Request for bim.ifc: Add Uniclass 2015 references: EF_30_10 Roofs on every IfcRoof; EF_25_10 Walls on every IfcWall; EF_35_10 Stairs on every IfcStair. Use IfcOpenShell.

First a look at what the model holds.

```python
import ifcopenshell

model = ifcopenshell.open("bim.ifc")
print(model.schema)
print("classifications:", [c.Name for c in model.by_type("IfcClassification")])
for ifc_class in ("IfcDoor", "IfcRoof", "IfcStair", "IfcWall", "IfcWindow"):
    print(ifc_class, len(model.by_type(ifc_class)))
```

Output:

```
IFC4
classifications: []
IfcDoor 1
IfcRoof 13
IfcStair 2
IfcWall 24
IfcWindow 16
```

```python
import ifcopenshell
import ifcopenshell.api.classification

model = ifcopenshell.open("bim.ifc")

system = ifcopenshell.api.classification.add_classification(model, classification="Uniclass 2015")

codes = {
    "IfcRoof": ("EF_30_10", "Roofs"),
    "IfcWall": ("EF_25_10", "Walls"),
    "IfcStair": ("EF_35_10", "Stairs"),
}
for ifc_class, (code, name) in codes.items():
    products = model.by_type(ifc_class)
    ifcopenshell.api.classification.add_reference(
        model, products=products, classification=system, identification=code, name=name
    )
    print(code, len(products))

model.write("bim-out.ifc")
```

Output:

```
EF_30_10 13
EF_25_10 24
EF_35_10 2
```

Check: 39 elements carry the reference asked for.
